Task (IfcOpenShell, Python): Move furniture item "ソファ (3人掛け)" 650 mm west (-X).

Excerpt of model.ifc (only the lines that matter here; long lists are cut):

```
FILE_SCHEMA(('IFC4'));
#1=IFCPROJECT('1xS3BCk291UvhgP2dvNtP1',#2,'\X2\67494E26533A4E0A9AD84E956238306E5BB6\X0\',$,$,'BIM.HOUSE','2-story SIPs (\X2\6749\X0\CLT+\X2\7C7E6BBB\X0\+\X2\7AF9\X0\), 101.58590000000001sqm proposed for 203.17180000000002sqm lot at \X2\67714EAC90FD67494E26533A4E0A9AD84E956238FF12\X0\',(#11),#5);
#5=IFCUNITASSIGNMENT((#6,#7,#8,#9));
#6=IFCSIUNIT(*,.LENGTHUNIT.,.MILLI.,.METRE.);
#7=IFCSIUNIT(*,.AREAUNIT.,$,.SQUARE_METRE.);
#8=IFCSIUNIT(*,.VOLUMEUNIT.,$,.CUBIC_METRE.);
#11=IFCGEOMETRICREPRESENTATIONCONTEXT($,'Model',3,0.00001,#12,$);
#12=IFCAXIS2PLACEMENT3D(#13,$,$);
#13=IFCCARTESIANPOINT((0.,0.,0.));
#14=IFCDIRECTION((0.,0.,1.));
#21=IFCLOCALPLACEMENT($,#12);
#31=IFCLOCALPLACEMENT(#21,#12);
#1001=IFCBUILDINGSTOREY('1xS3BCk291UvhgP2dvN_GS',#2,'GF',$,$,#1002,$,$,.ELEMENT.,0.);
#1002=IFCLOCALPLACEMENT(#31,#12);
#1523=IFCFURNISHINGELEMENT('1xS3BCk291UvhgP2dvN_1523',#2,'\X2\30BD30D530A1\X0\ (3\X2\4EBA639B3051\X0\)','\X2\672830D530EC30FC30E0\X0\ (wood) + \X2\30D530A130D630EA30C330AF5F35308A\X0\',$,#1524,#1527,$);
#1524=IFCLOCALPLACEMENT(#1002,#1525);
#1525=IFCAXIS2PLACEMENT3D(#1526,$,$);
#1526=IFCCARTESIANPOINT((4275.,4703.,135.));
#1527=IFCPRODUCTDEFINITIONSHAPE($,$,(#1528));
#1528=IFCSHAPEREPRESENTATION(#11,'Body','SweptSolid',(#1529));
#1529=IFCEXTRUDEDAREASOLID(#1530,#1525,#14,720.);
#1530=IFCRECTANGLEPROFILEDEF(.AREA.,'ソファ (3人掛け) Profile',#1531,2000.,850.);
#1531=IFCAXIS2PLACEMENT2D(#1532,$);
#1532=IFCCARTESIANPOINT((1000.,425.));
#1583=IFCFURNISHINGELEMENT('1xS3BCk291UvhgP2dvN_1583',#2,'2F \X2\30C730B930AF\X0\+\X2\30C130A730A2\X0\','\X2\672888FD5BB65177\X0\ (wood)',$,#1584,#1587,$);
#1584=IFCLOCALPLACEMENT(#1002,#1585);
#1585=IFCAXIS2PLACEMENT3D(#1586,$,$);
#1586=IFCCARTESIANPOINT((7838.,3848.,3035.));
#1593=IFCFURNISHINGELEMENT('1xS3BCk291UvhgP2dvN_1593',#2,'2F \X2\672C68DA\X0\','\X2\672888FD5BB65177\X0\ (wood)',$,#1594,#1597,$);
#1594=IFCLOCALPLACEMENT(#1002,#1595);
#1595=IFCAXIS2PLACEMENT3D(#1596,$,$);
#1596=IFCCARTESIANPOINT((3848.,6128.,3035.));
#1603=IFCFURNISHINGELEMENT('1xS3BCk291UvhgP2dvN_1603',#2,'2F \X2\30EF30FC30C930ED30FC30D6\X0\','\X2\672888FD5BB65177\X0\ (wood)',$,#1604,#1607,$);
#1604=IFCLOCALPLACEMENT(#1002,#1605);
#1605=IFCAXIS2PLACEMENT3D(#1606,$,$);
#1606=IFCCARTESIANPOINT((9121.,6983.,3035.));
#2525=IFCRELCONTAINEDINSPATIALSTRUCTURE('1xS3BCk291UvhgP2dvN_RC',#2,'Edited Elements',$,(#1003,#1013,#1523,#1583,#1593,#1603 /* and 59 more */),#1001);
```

```python
import ifcopenshell
import ifcopenshell.api.geometry
import ifcopenshell.util.placement

model = ifcopenshell.open("model.ifc")

item = model.by_guid("1xS3BCk291UvhgP2dvN_1523")
matrix = ifcopenshell.util.placement.get_local_placement(item.ObjectPlacement)
matrix[0, 3] -= 650.0
ifcopenshell.api.geometry.edit_object_placement(model, product=item, matrix=matrix, is_si=False)

print(ifcopenshell.util.placement.get_local_placement(item.ObjectPlacement).round(3) + 0.0)

model.write("model_updated.ifc")
```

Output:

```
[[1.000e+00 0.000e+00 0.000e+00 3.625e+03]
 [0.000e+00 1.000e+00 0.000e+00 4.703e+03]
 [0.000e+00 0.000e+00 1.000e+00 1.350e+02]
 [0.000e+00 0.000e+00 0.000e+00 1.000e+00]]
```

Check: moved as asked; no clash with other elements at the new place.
